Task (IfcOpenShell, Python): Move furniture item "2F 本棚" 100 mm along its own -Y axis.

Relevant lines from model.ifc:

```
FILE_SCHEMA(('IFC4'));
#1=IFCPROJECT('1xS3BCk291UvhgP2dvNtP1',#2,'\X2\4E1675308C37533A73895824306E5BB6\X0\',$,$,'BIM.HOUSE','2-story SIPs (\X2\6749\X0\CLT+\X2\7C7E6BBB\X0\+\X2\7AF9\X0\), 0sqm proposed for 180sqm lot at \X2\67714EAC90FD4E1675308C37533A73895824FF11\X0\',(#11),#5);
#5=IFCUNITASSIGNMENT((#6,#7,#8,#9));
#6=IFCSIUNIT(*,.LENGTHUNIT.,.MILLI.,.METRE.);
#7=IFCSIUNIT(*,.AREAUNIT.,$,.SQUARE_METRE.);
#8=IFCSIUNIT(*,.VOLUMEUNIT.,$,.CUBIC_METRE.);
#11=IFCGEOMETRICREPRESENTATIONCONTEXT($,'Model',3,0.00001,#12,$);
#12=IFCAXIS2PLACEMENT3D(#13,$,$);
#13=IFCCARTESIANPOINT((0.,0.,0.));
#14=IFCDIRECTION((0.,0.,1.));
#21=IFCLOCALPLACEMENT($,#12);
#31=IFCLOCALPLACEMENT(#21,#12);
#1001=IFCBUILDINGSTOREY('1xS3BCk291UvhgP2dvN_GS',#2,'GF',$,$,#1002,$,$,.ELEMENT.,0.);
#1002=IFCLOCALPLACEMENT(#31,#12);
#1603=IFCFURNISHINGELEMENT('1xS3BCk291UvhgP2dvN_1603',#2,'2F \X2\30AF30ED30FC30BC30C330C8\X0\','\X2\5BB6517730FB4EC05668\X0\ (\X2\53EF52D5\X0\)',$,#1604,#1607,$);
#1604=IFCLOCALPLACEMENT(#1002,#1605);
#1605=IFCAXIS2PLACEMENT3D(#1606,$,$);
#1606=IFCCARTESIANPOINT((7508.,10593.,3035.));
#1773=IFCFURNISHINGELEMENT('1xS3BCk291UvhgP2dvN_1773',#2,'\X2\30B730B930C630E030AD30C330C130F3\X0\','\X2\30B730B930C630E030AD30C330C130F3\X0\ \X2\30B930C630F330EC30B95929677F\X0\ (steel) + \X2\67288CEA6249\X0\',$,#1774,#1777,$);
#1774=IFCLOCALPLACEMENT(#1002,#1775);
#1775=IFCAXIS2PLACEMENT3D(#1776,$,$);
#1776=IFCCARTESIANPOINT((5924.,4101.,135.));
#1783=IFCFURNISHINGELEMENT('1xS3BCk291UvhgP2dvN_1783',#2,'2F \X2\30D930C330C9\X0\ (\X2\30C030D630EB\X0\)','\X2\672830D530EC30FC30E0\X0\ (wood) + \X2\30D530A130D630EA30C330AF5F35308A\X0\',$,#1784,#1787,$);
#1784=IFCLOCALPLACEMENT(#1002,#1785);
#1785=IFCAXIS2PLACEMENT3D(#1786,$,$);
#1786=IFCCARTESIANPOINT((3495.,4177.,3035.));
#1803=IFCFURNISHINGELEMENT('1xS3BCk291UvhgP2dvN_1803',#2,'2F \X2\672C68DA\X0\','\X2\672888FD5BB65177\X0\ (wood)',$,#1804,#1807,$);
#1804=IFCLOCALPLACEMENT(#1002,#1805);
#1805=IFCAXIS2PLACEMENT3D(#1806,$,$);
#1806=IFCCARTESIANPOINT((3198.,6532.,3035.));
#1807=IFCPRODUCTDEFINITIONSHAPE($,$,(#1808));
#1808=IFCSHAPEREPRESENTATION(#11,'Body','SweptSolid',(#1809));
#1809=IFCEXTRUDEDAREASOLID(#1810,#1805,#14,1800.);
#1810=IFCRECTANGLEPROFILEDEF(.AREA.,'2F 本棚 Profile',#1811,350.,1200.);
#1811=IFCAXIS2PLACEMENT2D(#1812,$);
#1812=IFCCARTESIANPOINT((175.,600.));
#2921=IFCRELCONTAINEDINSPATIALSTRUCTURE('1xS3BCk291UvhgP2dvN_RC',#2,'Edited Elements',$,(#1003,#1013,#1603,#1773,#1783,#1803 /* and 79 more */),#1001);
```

```python
import ifcopenshell
import ifcopenshell.api.geometry
import ifcopenshell.util.placement
import ifcopenshell.util.unit

model = ifcopenshell.open("model.ifc")
unit_scale = ifcopenshell.util.unit.calculate_unit_scale(model)

item = model.by_id(1803)
matrix = ifcopenshell.util.placement.get_local_placement(item.ObjectPlacement)
matrix[:3, 3] -= matrix[:3, 1] * 0.1 / unit_scale
ifcopenshell.api.geometry.edit_object_placement(model, product=item, matrix=matrix, is_si=False)

print(ifcopenshell.util.placement.get_local_placement(item.ObjectPlacement).round(3) + 0.0)

model.write("model_rev.ifc")
```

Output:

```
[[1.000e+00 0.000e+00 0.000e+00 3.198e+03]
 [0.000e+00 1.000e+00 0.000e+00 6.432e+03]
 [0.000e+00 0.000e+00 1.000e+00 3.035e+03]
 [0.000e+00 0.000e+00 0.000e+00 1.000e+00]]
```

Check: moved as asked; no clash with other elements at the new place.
